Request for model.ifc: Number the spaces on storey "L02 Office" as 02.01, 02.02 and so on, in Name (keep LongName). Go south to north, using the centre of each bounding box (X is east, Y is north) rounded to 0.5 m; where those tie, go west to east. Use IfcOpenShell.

First a look at what the model holds.

```python
import ifcopenshell
import ifcopenshell.util.element
import ifcopenshell.util.placement

model = ifcopenshell.open("model.ifc")
print(model.schema)
storey = next(s for s in model.by_type("IfcBuildingStorey") if s.Name == "L02 Office")
spaces = [e for e in ifcopenshell.util.element.get_decomposition(storey) if e.is_a("IfcSpace")]
for e in sorted(spaces, key=lambda e: e.id()):
    origin = ifcopenshell.util.placement.get_local_placement(e.ObjectPlacement)[:3, 3]
    print(e.id(), e.Name, e.LongName, origin.round(2) + 0.0, sep=" | ")
```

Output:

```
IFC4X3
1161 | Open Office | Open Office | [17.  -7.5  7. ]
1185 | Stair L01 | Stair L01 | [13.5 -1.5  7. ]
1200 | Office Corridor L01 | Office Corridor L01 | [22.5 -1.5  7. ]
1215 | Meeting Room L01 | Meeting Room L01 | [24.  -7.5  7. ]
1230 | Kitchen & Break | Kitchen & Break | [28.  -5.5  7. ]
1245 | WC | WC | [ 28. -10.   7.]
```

```python
import ifcopenshell
import ifcopenshell.geom
import ifcopenshell.util.element
import ifcopenshell.util.shape

model = ifcopenshell.open("model.ifc")
settings = ifcopenshell.geom.settings()
settings.set("use-world-coords", True)


def centre(element):
    shape = ifcopenshell.geom.create_shape(settings, element)
    return ifcopenshell.util.shape.get_bbox_centroid(shape.geometry)


storey = next(s for s in model.by_type("IfcBuildingStorey") if s.Name == "L02 Office")
spaces = [e for e in ifcopenshell.util.element.get_decomposition(storey) if e.is_a("IfcSpace")]

# Insertion points can sit at a corner or the storey origin, so sort by the geometry (in metres).
centres = {e: centre(e) for e in spaces}
spaces.sort(key=lambda e: (round(centres[e][1] / 0.5), centres[e][0]))

for i, e in enumerate(spaces, start=1):
    number = f"02.{i:02d}"
    e.Name = number
    print(e.id(), number)

model.write("model_updated.ifc")
```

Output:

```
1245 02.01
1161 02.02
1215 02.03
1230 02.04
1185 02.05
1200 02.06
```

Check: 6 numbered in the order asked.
